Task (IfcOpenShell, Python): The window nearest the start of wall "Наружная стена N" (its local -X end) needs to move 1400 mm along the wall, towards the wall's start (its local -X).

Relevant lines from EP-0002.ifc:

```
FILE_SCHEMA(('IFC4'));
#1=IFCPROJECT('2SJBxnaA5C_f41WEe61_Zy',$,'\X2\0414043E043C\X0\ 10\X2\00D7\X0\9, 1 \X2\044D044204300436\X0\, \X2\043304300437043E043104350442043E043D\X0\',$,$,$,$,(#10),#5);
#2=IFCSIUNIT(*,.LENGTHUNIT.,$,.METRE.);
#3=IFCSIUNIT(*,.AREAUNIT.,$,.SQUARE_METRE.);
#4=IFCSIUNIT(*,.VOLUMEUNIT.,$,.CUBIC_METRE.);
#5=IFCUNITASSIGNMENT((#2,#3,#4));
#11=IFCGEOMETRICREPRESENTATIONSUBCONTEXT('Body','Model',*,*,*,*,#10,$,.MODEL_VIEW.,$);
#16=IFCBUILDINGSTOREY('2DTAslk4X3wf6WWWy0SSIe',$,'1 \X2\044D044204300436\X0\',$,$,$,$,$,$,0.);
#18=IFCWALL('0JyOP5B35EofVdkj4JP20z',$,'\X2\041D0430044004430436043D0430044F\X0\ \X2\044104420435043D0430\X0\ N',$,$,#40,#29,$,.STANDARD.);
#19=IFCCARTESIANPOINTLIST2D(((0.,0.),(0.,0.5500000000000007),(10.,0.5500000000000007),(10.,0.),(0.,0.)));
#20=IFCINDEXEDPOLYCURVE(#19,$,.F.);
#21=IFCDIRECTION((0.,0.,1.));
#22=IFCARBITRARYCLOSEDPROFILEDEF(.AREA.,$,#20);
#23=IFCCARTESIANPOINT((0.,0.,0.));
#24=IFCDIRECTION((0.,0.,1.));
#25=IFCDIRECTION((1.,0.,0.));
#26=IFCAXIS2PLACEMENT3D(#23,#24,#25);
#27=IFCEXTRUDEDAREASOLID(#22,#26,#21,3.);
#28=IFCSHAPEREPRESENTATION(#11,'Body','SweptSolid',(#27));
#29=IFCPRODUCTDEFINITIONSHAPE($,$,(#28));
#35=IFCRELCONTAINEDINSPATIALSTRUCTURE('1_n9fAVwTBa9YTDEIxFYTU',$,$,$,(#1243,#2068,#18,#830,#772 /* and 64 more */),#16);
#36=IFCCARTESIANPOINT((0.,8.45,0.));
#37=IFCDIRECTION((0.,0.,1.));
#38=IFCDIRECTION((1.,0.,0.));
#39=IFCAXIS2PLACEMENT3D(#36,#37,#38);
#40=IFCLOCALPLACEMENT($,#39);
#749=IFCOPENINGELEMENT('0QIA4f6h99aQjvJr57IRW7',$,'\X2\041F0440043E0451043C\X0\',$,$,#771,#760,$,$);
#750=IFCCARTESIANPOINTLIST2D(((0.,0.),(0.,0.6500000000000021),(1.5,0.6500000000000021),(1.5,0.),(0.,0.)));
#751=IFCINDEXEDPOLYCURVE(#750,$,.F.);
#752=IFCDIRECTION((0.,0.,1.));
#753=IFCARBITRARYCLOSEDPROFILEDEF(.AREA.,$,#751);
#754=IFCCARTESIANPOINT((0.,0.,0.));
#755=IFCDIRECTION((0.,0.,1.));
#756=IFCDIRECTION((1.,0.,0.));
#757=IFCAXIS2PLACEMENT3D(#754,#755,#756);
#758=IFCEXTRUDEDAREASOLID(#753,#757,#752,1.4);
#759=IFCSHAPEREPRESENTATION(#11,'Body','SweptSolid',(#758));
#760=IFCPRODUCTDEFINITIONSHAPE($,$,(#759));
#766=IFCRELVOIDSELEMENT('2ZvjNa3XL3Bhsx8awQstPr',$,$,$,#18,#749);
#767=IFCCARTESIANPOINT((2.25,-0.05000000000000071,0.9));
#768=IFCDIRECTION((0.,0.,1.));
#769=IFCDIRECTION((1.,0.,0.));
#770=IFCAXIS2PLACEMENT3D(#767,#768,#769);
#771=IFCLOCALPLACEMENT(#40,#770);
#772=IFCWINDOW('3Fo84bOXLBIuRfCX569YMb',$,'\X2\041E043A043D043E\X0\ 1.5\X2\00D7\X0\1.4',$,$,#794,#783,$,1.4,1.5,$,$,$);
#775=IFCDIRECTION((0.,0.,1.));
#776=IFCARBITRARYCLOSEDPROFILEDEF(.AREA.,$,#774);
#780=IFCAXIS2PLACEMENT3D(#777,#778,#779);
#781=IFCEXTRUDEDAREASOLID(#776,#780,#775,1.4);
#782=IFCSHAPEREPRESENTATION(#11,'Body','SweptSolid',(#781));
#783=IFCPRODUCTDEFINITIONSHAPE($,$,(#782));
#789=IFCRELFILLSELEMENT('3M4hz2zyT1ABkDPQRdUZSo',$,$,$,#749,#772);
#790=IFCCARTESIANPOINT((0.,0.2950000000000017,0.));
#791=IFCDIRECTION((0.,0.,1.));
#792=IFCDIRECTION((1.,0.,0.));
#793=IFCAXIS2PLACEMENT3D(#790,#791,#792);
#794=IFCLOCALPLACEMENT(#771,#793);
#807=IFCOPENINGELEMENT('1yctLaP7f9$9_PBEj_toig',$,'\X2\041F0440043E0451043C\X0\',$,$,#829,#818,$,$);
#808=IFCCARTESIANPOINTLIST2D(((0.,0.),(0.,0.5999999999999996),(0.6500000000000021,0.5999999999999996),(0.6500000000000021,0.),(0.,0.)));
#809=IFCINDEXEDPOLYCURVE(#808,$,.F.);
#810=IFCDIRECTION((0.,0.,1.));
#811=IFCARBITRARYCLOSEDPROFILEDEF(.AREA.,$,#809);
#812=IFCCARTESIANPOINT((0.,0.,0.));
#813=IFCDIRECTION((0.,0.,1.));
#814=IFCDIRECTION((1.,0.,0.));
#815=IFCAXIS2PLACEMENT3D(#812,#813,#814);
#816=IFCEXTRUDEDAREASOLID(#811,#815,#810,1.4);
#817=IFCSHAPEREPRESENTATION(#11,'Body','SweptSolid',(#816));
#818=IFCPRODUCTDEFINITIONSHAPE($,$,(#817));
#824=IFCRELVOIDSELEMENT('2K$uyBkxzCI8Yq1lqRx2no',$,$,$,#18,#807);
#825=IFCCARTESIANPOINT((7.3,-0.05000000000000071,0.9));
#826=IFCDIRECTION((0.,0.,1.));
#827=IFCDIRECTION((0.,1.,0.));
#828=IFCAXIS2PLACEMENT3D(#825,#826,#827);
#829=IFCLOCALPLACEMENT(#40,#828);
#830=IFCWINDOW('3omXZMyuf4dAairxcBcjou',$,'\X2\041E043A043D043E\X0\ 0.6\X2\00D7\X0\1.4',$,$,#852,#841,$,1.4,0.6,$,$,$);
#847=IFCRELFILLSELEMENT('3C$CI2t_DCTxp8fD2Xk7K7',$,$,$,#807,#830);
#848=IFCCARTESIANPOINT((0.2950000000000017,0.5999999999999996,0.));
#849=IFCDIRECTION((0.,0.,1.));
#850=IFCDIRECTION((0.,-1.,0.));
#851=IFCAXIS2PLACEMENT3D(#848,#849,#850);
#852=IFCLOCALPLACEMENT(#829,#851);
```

```python
import ifcopenshell
import ifcopenshell.api.geometry
import ifcopenshell.util.placement

model = ifcopenshell.open("EP-0002.ifc")

window = model.by_guid("3Fo84bOXLBIuRfCX569YMb")
opening = window.FillsVoids[0].RelatingOpeningElement
wall = opening.VoidsElements[0].RelatingBuildingElement

wall_matrix = ifcopenshell.util.placement.get_local_placement(wall.ObjectPlacement)
shift = wall_matrix[:3, 0] * -1.4
before = ifcopenshell.util.placement.get_local_placement(window.ObjectPlacement)[:3, 3].copy()

# The window is placed relative to its opening, so it follows when the opening moves.
matrix = ifcopenshell.util.placement.get_local_placement(opening.ObjectPlacement)
matrix[:3, 3] += shift
ifcopenshell.api.geometry.edit_object_placement(
    model, product=opening, matrix=matrix, is_si=False, should_transform_children=True
)

after = ifcopenshell.util.placement.get_local_placement(window.ObjectPlacement)[:3, 3]
print("window moved by", (after - before).round(3) + 0.0)

model.write("EP-0002_updated.ifc")
```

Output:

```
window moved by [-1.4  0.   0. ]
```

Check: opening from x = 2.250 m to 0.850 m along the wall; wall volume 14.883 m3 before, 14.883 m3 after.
